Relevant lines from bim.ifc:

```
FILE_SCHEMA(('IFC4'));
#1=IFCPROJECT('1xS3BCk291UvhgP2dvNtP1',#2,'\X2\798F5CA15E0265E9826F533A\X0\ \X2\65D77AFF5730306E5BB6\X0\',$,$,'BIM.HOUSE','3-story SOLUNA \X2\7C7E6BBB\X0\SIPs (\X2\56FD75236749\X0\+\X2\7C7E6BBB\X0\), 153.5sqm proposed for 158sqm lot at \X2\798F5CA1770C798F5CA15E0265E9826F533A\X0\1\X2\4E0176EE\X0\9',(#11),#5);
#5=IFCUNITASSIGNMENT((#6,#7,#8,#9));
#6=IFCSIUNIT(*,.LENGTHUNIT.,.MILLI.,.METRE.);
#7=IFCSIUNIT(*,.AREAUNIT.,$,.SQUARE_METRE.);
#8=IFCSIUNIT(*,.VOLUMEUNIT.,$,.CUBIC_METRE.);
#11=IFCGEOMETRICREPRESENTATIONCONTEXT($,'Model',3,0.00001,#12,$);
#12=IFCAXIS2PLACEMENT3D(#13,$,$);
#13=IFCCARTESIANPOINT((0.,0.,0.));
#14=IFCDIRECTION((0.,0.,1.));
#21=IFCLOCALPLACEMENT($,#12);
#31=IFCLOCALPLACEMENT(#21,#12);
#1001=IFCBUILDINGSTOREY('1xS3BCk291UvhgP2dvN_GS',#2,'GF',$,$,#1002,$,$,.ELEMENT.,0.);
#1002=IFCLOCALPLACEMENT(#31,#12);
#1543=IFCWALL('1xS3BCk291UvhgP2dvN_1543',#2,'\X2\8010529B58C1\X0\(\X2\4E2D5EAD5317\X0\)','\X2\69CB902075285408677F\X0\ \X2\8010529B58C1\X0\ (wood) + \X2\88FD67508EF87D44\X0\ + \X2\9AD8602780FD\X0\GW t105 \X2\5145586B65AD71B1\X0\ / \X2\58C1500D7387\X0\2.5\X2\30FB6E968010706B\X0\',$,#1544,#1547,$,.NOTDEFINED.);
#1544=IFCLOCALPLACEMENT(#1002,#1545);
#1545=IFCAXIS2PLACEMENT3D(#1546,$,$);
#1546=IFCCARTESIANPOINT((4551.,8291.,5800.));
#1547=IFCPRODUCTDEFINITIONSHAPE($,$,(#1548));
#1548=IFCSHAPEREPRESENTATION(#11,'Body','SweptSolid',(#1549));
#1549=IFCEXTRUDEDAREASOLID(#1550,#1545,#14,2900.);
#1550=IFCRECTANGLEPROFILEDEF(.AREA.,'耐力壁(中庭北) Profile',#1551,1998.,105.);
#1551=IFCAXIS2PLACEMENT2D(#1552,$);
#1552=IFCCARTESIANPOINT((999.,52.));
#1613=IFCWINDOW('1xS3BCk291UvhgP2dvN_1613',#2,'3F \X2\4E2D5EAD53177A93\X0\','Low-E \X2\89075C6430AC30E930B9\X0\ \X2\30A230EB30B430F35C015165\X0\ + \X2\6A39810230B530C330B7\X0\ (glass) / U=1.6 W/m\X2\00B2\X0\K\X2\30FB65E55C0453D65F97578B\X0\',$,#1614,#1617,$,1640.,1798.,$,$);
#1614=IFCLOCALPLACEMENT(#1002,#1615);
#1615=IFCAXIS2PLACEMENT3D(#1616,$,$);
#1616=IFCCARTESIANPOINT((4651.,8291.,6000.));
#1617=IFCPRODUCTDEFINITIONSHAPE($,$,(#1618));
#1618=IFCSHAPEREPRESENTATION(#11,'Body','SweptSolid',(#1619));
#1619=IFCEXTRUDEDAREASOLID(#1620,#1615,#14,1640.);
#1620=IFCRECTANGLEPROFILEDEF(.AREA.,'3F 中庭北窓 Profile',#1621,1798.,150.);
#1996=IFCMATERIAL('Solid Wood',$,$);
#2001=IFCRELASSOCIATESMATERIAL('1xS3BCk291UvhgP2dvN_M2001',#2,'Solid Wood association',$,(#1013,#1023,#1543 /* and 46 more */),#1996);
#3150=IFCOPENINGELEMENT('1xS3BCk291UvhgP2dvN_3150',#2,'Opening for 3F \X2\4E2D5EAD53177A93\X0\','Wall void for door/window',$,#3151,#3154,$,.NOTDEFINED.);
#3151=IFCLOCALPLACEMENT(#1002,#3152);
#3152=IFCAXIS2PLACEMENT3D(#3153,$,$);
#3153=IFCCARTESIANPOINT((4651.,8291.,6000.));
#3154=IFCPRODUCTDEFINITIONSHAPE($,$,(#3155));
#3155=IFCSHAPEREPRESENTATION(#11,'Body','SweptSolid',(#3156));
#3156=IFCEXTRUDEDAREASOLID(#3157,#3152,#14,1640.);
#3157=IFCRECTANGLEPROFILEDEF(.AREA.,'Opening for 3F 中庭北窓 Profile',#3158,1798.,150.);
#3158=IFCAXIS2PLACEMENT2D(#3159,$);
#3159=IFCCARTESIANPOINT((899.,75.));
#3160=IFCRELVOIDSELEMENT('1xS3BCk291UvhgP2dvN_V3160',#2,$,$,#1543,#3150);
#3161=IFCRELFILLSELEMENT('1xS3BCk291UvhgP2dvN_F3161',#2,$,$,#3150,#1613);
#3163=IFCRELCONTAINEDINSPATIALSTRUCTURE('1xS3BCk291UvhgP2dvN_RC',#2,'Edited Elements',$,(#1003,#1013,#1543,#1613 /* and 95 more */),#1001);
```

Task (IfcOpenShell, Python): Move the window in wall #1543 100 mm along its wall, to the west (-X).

```python
import ifcopenshell
import ifcopenshell.api.geometry
import ifcopenshell.util.placement

model = ifcopenshell.open("bim.ifc")

window = model.by_id(1613)
opening = window.FillsVoids[0].RelatingOpeningElement
wall = opening.VoidsElements[0].RelatingBuildingElement

wall_matrix = ifcopenshell.util.placement.get_local_placement(wall.ObjectPlacement)
shift = wall_matrix[:3, 0] * -100.0
before = ifcopenshell.util.placement.get_local_placement(window.ObjectPlacement)[:3, 3].copy()

# The window is not placed relative to its opening, so move both.
for product in (opening, window):
    matrix = ifcopenshell.util.placement.get_local_placement(product.ObjectPlacement)
    matrix[:3, 3] += shift
    ifcopenshell.api.geometry.edit_object_placement(model, product=product, matrix=matrix, is_si=False)

after = ifcopenshell.util.placement.get_local_placement(window.ObjectPlacement)[:3, 3]
print("window moved by", (after - before).round(3) + 0.0)

model.write("bim_edited.ifc")
```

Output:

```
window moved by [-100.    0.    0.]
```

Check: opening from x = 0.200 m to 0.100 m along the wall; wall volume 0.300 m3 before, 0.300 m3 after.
